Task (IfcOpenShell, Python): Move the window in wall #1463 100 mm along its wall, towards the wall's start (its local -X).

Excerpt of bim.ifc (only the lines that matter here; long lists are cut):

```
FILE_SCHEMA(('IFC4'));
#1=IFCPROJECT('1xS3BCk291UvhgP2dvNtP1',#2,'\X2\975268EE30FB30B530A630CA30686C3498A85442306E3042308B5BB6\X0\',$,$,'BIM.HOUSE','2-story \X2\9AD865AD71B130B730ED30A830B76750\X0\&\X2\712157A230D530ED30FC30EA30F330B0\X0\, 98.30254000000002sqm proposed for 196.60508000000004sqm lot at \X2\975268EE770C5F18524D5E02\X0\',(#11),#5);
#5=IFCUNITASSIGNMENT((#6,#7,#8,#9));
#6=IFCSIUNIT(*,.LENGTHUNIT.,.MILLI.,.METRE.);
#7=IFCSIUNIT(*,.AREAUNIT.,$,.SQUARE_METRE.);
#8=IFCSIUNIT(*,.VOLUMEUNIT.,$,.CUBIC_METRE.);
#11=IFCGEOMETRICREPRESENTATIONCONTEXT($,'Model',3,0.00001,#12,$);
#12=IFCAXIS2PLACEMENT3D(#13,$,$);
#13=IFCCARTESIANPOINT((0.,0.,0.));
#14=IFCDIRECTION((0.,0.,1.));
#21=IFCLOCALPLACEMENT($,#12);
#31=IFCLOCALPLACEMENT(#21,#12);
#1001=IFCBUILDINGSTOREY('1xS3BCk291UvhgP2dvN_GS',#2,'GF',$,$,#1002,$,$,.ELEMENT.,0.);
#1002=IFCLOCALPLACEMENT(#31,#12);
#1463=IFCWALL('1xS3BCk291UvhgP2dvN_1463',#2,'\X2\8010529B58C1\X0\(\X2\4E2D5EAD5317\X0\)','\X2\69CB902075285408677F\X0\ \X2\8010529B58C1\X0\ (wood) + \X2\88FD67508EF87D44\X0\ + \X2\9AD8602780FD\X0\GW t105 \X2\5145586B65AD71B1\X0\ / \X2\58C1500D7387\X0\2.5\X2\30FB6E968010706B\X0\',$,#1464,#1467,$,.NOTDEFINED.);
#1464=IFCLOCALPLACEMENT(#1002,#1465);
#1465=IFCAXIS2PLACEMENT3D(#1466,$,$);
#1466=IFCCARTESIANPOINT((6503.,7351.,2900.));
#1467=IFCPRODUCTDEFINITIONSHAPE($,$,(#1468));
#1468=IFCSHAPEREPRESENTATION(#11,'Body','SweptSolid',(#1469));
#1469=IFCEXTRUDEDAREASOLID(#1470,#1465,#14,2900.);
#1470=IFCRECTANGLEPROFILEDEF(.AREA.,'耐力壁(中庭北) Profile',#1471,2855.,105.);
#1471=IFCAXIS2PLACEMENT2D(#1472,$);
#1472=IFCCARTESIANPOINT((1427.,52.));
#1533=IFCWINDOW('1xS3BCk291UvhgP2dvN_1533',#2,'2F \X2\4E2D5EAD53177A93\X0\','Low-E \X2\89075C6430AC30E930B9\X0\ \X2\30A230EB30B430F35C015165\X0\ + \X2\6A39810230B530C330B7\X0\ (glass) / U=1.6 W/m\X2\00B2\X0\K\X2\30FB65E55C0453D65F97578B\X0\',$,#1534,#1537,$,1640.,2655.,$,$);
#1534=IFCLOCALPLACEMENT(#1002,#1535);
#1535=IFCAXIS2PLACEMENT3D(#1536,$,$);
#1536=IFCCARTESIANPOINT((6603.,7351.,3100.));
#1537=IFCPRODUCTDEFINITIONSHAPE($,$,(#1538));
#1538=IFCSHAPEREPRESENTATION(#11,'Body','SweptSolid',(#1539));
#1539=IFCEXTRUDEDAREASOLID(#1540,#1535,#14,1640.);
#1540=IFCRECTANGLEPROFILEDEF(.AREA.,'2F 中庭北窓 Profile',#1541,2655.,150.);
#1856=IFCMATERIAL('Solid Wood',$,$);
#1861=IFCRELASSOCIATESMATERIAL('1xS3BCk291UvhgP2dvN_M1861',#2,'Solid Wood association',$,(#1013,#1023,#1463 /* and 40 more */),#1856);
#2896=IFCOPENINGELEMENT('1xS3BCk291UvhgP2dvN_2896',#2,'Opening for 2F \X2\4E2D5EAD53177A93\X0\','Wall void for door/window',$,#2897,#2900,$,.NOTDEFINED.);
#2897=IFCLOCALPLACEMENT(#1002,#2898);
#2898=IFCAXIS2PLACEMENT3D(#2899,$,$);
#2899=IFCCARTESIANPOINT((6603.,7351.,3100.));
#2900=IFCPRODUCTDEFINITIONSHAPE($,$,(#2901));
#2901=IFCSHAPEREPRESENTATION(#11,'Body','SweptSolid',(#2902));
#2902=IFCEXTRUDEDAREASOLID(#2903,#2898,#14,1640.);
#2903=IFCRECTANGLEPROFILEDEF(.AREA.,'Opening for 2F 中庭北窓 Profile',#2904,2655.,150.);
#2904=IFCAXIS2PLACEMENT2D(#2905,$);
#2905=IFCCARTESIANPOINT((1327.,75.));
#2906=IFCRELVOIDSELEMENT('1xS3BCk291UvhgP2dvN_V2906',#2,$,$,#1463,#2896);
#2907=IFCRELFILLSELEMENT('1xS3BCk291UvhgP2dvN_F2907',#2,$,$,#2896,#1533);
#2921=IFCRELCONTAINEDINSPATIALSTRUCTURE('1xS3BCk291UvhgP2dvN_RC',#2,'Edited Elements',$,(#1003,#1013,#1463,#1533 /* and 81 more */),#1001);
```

```python
import ifcopenshell
import ifcopenshell.api.geometry
import ifcopenshell.util.placement

model = ifcopenshell.open("bim.ifc")

window = model.by_id(1533)
opening = window.FillsVoids[0].RelatingOpeningElement
wall = opening.VoidsElements[0].RelatingBuildingElement

wall_matrix = ifcopenshell.util.placement.get_local_placement(wall.ObjectPlacement)
shift = wall_matrix[:3, 0] * -100.0
before = ifcopenshell.util.placement.get_local_placement(window.ObjectPlacement)[:3, 3].copy()

# The window is not placed relative to its opening, so move both.
for product in (opening, window):
    matrix = ifcopenshell.util.placement.get_local_placement(product.ObjectPlacement)
    matrix[:3, 3] += shift
    ifcopenshell.api.geometry.edit_object_placement(model, product=product, matrix=matrix, is_si=False)

after = ifcopenshell.util.placement.get_local_placement(window.ObjectPlacement)[:3, 3]
print("window moved by", (after - before).round(3) + 0.0)

model.write("bim_rev.ifc")
```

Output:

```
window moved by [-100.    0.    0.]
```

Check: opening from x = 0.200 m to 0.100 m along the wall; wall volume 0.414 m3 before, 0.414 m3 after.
